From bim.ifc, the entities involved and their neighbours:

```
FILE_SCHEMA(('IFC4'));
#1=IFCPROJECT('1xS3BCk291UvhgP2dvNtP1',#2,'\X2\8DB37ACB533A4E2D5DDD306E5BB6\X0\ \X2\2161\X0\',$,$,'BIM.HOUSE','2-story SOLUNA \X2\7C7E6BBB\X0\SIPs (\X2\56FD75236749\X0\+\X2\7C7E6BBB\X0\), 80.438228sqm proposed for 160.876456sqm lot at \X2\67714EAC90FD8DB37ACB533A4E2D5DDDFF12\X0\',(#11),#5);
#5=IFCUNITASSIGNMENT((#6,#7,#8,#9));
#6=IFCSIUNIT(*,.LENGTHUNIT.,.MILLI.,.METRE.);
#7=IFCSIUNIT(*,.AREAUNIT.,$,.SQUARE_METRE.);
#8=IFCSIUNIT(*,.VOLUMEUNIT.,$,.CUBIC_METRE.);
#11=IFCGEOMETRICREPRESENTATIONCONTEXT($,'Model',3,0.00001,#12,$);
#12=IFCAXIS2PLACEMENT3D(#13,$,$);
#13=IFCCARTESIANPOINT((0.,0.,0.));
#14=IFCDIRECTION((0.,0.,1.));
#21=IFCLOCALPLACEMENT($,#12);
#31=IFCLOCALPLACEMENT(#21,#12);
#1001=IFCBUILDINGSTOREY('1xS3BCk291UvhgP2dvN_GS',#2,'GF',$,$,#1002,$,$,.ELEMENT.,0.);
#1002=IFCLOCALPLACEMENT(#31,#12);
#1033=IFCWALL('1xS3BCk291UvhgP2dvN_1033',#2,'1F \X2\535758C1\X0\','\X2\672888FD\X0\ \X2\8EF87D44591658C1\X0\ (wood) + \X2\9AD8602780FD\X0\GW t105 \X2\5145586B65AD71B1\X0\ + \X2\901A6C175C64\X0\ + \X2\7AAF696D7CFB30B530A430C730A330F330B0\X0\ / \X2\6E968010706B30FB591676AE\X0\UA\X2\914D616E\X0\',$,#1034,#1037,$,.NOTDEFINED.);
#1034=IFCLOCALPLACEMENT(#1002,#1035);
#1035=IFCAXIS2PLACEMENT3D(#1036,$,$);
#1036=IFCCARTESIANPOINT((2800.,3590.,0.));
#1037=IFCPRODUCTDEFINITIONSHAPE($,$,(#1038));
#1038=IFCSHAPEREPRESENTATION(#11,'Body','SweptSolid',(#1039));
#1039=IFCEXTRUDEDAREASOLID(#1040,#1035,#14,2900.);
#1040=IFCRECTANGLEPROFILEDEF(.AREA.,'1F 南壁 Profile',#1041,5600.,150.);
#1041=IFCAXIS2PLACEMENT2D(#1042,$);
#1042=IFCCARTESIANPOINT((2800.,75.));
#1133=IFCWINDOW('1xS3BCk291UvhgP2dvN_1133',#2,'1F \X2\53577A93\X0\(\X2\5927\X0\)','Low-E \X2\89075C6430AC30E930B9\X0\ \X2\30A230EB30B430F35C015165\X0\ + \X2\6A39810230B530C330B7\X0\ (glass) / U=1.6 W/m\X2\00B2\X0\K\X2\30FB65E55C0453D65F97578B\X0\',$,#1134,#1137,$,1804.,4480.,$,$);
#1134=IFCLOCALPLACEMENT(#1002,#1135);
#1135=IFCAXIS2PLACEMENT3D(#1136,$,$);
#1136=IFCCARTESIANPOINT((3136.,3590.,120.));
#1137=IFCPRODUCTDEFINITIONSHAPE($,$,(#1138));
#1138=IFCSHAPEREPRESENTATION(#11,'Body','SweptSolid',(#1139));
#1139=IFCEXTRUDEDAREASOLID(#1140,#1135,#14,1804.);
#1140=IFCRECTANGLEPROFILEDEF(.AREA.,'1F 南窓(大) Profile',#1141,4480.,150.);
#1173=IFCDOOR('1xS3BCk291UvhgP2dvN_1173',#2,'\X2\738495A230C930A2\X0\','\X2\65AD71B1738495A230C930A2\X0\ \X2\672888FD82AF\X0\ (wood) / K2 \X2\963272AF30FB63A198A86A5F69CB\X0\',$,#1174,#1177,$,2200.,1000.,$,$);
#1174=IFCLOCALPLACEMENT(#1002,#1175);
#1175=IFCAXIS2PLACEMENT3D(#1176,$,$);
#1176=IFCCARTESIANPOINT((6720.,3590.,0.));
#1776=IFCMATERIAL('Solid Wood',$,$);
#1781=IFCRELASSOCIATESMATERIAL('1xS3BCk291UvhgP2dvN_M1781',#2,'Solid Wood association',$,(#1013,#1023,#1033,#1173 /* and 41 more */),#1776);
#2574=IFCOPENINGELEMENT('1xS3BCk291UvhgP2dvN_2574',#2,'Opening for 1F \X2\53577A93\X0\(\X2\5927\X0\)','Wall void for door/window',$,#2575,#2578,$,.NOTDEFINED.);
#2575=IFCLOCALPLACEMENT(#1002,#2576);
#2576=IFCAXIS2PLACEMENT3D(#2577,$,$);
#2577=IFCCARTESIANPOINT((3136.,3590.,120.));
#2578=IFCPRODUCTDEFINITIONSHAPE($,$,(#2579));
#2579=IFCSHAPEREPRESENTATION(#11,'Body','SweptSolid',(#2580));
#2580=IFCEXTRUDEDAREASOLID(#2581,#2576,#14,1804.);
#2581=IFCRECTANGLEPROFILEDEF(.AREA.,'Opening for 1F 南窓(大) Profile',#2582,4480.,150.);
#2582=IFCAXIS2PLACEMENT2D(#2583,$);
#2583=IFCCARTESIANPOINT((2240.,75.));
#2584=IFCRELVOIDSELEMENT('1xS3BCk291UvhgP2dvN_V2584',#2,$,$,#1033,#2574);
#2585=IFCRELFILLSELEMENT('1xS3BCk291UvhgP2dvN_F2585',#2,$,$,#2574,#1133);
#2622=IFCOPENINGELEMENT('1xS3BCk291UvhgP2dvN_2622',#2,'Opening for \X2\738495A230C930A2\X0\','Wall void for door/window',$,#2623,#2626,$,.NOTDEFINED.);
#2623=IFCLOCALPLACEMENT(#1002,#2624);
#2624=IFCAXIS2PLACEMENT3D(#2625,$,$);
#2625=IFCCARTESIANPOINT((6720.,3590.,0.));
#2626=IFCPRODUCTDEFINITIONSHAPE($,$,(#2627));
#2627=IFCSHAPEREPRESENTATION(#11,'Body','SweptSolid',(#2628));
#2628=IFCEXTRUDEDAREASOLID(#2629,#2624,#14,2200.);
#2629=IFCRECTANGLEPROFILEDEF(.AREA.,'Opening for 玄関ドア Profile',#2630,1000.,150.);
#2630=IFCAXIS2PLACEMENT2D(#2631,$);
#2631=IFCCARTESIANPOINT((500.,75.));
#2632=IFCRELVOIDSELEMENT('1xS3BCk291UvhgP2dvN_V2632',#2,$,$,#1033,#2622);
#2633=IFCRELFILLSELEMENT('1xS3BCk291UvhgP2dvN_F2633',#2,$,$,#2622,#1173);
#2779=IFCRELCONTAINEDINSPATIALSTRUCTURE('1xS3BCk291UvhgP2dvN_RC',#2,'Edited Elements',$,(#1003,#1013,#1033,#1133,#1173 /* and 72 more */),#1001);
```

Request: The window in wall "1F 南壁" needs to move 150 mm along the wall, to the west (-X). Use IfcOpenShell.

```python
import ifcopenshell
import ifcopenshell.api.geometry
import ifcopenshell.util.placement
import ifcopenshell.util.unit

model = ifcopenshell.open("bim.ifc")
unit_scale = ifcopenshell.util.unit.calculate_unit_scale(model)

window = model.by_id(1133)
opening = window.FillsVoids[0].RelatingOpeningElement
wall = opening.VoidsElements[0].RelatingBuildingElement

wall_matrix = ifcopenshell.util.placement.get_local_placement(wall.ObjectPlacement)
shift = wall_matrix[:3, 0] * -0.15 / unit_scale
before = ifcopenshell.util.placement.get_local_placement(window.ObjectPlacement)[:3, 3].copy()

# The window is not placed relative to its opening, so move both.
for product in (opening, window):
    matrix = ifcopenshell.util.placement.get_local_placement(product.ObjectPlacement)
    matrix[:3, 3] += shift
    ifcopenshell.api.geometry.edit_object_placement(model, product=product, matrix=matrix, is_si=False)

after = ifcopenshell.util.placement.get_local_placement(window.ObjectPlacement)[:3, 3]
print("window moved by", (after - before).round(3) + 0.0)

model.write("bim_edited.ifc")
```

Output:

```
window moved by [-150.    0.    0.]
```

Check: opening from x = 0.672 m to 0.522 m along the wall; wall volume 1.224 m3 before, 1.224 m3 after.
